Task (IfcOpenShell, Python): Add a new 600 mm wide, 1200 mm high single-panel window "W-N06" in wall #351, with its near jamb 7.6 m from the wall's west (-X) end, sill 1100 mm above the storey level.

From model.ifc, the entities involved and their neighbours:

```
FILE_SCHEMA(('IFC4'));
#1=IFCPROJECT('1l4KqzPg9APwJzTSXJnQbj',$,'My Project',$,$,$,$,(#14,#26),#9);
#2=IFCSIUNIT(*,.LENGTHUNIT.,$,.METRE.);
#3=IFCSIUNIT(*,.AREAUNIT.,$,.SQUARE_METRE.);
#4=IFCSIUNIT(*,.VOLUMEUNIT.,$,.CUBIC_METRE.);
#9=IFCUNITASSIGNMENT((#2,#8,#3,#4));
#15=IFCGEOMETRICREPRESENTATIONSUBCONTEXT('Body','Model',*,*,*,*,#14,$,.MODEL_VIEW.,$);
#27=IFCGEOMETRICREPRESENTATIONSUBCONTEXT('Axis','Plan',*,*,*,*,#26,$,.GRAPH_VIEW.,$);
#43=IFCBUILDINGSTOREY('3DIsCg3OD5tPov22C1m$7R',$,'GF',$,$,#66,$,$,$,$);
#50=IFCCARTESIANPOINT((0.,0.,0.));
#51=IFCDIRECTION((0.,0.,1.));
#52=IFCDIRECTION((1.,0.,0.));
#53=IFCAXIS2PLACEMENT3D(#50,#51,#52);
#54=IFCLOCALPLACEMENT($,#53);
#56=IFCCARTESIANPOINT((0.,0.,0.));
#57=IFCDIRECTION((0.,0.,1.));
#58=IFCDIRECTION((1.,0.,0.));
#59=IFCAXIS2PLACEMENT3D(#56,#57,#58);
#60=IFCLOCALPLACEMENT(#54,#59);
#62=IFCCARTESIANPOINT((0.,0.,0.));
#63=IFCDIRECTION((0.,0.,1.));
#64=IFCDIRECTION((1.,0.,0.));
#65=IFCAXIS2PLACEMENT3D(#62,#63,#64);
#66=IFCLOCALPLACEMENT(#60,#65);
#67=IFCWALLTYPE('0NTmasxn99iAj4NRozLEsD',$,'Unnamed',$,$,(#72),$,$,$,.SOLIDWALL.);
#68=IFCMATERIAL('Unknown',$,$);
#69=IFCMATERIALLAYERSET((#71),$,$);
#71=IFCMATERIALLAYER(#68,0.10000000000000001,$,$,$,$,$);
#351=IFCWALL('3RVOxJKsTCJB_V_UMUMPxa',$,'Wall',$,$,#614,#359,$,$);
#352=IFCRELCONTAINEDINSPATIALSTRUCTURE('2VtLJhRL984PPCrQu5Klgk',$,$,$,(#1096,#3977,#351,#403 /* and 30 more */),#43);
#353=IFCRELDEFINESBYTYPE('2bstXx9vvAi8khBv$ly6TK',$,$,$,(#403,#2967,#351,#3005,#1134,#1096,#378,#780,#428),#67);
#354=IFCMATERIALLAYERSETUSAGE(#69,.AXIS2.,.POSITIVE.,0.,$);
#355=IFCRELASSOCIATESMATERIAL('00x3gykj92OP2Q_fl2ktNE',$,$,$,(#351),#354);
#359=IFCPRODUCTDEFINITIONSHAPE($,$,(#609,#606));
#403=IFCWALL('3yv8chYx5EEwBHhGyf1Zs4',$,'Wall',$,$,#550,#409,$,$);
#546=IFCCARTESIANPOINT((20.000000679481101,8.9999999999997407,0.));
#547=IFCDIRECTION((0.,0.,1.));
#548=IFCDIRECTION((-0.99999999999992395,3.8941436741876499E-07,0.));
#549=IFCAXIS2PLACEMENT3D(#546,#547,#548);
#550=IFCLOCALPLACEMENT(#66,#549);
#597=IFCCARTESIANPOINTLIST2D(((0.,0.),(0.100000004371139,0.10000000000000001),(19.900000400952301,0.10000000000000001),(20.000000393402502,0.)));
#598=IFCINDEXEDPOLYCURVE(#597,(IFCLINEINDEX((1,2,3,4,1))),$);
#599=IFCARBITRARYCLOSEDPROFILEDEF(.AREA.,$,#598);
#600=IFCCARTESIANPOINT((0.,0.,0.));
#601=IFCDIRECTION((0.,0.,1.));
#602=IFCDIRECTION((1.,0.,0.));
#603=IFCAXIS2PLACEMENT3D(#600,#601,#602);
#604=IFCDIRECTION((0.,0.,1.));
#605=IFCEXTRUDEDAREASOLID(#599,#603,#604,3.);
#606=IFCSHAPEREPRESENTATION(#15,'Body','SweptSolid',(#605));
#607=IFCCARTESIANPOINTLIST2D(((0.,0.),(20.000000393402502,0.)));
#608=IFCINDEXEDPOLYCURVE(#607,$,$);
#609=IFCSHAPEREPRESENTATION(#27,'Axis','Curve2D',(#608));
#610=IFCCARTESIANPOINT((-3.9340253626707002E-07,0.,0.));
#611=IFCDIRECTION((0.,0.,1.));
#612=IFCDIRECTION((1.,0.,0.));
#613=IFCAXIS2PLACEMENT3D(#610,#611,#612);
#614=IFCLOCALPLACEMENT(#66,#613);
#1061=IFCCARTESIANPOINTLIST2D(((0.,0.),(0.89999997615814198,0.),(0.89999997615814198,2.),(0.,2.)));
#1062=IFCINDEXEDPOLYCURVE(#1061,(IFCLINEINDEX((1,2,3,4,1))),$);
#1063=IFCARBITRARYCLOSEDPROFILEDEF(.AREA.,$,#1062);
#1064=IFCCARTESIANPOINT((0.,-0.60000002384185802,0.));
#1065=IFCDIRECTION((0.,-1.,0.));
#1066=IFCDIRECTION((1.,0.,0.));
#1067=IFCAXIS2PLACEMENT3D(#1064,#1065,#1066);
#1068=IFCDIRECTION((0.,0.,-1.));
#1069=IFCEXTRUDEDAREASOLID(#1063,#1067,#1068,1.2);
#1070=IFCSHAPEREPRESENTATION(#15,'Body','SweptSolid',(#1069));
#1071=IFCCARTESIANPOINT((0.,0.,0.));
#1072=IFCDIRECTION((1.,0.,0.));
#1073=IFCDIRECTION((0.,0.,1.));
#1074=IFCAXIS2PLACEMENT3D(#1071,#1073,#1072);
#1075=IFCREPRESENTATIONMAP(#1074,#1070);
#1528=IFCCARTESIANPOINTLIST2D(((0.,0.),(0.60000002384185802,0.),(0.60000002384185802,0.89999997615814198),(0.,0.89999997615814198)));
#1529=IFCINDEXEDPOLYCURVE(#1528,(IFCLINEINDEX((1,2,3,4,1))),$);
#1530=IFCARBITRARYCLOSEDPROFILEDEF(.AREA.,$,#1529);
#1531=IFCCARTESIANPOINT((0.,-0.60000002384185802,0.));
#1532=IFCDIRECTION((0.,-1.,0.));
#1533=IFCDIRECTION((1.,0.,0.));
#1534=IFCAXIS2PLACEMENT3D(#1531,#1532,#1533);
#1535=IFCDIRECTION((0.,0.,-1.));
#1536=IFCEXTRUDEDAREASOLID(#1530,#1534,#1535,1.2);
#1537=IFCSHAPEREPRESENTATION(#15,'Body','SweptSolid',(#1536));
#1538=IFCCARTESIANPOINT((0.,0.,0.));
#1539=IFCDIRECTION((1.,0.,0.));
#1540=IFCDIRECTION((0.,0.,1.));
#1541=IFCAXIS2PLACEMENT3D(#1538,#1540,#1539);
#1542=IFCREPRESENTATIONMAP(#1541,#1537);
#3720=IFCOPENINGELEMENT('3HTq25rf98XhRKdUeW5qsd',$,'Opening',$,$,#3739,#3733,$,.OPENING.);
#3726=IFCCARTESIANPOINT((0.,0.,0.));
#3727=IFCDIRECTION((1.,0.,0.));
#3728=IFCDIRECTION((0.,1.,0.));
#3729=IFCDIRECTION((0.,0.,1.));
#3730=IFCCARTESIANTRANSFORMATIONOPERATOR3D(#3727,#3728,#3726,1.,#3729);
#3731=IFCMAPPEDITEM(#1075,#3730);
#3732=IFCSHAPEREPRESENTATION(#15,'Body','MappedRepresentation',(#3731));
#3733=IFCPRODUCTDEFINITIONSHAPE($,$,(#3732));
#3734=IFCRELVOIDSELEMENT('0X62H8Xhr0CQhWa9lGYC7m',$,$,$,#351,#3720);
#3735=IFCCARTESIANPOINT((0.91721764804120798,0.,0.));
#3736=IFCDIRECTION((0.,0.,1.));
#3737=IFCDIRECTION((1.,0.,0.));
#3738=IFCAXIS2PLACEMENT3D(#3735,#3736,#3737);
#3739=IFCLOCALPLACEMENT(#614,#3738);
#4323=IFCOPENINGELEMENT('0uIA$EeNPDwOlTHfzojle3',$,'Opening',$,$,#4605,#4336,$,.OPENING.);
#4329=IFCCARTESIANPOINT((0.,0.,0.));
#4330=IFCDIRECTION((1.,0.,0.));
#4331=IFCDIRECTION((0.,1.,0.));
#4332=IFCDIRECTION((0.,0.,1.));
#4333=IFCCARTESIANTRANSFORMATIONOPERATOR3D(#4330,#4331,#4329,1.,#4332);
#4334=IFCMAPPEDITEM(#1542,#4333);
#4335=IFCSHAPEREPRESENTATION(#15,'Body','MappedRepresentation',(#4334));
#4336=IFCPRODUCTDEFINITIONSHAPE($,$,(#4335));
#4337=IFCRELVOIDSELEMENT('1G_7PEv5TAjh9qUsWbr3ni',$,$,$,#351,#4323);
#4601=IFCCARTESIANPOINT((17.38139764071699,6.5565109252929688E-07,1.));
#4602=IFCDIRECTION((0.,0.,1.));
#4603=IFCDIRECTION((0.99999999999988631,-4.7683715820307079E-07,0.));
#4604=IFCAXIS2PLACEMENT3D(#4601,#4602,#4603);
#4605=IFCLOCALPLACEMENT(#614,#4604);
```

```python
import numpy as np
import ifcopenshell
import ifcopenshell.api.feature
import ifcopenshell.api.geometry
import ifcopenshell.api.root
import ifcopenshell.api.spatial
import ifcopenshell.geom
import ifcopenshell.util.element
import ifcopenshell.util.placement
import ifcopenshell.util.representation
import ifcopenshell.util.shape
import ifcopenshell.util.unit

model = ifcopenshell.open("model.ifc")
unit_scale = ifcopenshell.util.unit.calculate_unit_scale(model)
settings = ifcopenshell.geom.settings()


def volume(element):
    """Net volume in cubic metres, openings subtracted."""
    shape = ifcopenshell.geom.create_shape(settings, element)
    return ifcopenshell.util.shape.get_volume(shape.geometry)


wall = model.by_id(351)
storey = ifcopenshell.util.element.get_container(wall, ifc_class="IfcBuildingStorey")
context = ifcopenshell.util.representation.get_context(model, "Model", "Body", "MODEL_VIEW")
before = volume(wall)

width, height, from_end, sill = 0.6, 1.2, 7.6, 1.1  # metres

# The wall runs along its own X axis, and the end named is its -X end.
wall_shape = ifcopenshell.geom.create_shape(settings, wall)
x, y, z = ifcopenshell.util.shape.get_vertices(wall_shape.geometry).T
start = x.min() + from_end
face, thickness = float(y.min()), float(y.max() - y.min())
wall_matrix = ifcopenshell.util.placement.get_local_placement(wall.ObjectPlacement)
level = ifcopenshell.util.placement.get_local_placement(storey.ObjectPlacement)[2, 3]


def in_wall(x, y):
    """Placement at x, y metres in the wall's axes, at sill height."""
    matrix = wall_matrix.copy()
    matrix[:, 3] = wall_matrix @ np.array([x / unit_scale, y / unit_scale, 0.0, 1.0])
    matrix[2, 3] = level + sill / unit_scale
    return matrix


# Opening: a box that overshoots both wall faces by 50 mm.
opening = ifcopenshell.api.root.create_entity(model, ifc_class="IfcOpeningElement", predefined_type="OPENING")
box = ifcopenshell.api.geometry.add_wall_representation(
    model, context=context, length=width, height=height, thickness=thickness + 0.1
)
ifcopenshell.api.geometry.assign_representation(model, product=opening, representation=box)
ifcopenshell.api.geometry.edit_object_placement(model, product=opening, matrix=in_wall(start, face - 0.05), is_si=False)
ifcopenshell.api.feature.add_feature(model, feature=opening, element=wall)

window = ifcopenshell.api.root.create_entity(model, ifc_class="IfcWindow", name="W-N06", predefined_type="WINDOW")
window.OverallWidth, window.OverallHeight = width / unit_scale, height / unit_scale
window.PartitioningType = "SINGLE_PANEL"
body = ifcopenshell.api.geometry.add_window_representation(
    model,
    context=context,
    overall_width=window.OverallWidth,
    overall_height=window.OverallHeight,
    partition_type="SINGLE_PANEL",
)
ifcopenshell.api.geometry.assign_representation(model, product=window, representation=body)
ifcopenshell.api.spatial.assign_container(model, products=[window], relating_structure=storey)
ifcopenshell.api.feature.add_filling(model, opening=opening, element=window)

# Centre the window in the wall's thickness.
ifcopenshell.api.geometry.edit_object_placement(model, product=window, matrix=in_wall(start, face), is_si=False)
window_shape = ifcopenshell.geom.create_shape(settings, window)
depth = ifcopenshell.util.shape.get_vertices(window_shape.geometry)[:, 1]
offset = face + thickness / 2 - (depth.min() + depth.max()) / 2
ifcopenshell.api.geometry.edit_object_placement(model, product=window, matrix=in_wall(start, offset), is_si=False)

after = volume(wall)

print(f"wall volume {before:.3f} -> {after:.3f} m3")

model.write("model_edited.ifc")
```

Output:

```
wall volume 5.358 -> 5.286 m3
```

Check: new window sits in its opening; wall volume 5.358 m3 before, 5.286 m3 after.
